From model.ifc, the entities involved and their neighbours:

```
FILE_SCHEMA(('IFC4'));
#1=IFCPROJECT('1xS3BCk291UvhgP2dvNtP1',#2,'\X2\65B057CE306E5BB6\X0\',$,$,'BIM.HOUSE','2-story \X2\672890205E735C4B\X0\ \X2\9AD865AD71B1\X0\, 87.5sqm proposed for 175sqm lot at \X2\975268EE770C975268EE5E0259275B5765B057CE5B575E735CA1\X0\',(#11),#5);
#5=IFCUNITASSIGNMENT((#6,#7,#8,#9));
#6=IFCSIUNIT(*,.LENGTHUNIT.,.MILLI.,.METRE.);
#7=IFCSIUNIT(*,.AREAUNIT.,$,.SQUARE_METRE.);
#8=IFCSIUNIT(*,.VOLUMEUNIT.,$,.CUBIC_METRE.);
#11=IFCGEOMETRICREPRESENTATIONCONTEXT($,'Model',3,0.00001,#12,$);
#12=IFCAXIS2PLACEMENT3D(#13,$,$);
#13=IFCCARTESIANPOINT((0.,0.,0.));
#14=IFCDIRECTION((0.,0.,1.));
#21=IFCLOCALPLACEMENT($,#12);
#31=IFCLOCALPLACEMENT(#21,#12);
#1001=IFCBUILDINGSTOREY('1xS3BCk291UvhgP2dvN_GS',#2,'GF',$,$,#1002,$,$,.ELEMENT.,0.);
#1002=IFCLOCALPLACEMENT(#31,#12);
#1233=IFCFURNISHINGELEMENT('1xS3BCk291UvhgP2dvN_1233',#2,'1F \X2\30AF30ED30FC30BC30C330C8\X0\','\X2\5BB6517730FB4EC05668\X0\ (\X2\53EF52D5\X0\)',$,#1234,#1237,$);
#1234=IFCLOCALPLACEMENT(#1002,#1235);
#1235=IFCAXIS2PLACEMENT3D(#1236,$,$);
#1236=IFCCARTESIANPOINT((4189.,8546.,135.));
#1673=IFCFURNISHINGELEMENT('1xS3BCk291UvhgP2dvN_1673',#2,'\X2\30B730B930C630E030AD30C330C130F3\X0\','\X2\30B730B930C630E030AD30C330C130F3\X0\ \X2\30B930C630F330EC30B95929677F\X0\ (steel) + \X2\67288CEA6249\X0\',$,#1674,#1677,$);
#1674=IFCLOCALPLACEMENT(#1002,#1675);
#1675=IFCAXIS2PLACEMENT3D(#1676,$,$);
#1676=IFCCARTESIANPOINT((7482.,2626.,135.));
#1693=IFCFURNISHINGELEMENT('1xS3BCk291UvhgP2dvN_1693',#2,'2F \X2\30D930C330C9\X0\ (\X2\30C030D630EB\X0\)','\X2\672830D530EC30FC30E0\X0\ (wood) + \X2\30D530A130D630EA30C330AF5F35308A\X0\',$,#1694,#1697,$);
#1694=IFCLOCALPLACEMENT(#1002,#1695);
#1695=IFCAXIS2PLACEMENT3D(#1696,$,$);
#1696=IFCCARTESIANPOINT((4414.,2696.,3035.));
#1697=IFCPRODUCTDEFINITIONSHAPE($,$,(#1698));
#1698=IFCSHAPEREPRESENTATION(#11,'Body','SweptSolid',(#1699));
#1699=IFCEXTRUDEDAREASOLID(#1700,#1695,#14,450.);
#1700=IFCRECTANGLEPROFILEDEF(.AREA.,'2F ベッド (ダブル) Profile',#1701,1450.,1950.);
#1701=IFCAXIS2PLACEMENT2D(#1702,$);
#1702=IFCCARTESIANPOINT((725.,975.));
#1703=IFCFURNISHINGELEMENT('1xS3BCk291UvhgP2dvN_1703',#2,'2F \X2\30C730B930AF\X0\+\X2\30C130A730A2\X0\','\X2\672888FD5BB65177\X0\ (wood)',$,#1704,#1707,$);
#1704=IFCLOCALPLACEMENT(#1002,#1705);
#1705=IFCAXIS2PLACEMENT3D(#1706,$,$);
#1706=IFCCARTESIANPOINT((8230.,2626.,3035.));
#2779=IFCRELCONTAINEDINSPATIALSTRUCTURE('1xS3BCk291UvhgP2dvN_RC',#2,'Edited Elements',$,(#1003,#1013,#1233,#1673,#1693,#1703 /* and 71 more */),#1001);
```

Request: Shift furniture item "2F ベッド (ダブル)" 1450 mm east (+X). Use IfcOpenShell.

```python
import ifcopenshell
import ifcopenshell.api.geometry
import ifcopenshell.util.placement
import ifcopenshell.util.unit

model = ifcopenshell.open("model.ifc")
unit_scale = ifcopenshell.util.unit.calculate_unit_scale(model)

item = model.by_id(1693)
matrix = ifcopenshell.util.placement.get_local_placement(item.ObjectPlacement)
matrix[0, 3] += 1.45 / unit_scale
ifcopenshell.api.geometry.edit_object_placement(model, product=item, matrix=matrix, is_si=False)

print(ifcopenshell.util.placement.get_local_placement(item.ObjectPlacement).round(3) + 0.0)

model.write("model_v2.ifc")
```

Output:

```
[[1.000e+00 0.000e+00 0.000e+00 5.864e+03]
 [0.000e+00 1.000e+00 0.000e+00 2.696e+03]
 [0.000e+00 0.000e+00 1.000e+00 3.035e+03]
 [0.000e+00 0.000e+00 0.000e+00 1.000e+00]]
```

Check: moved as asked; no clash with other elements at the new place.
